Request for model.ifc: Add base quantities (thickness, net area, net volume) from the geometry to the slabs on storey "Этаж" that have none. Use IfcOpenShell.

First a look at what the model holds.

```python
import ifcopenshell
import ifcopenshell.util.element
import ifcopenshell.util.unit

model = ifcopenshell.open("model.ifc")
print(model.schema)
for unit_type in ("LENGTHUNIT", "AREAUNIT", "VOLUMEUNIT"):
    print(unit_type, ifcopenshell.util.unit.calculate_unit_scale(model, unit_type))
storey = next(s for s in model.by_type("IfcBuildingStorey") if s.Name == "Этаж")
slabs = [e for e in ifcopenshell.util.element.get_decomposition(storey) if e.is_a("IfcSlab")]
for e in sorted(slabs, key=lambda e: e.id()):
    print(e.id(), e.is_a(), e.Name, list(ifcopenshell.util.element.get_psets(e, qtos_only=True)), sep=" | ")
```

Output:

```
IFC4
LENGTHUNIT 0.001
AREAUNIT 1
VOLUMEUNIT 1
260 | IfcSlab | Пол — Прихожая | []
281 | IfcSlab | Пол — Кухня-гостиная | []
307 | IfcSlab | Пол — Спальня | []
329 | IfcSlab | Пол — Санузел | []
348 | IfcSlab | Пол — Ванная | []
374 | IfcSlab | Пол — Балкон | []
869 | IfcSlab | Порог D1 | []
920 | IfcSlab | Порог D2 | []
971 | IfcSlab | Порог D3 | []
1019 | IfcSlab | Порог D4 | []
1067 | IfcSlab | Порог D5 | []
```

```python
import ifcopenshell
import ifcopenshell.api.pset
import ifcopenshell.geom
import ifcopenshell.util.element
import ifcopenshell.util.shape
import ifcopenshell.util.unit

model = ifcopenshell.open("model.ifc")
unit_scale = ifcopenshell.util.unit.calculate_unit_scale(model)
area_scale = ifcopenshell.util.unit.calculate_unit_scale(model, "AREAUNIT")
volume_scale = ifcopenshell.util.unit.calculate_unit_scale(model, "VOLUMEUNIT")
settings = ifcopenshell.geom.settings()

storey = next(s for s in model.by_type("IfcBuildingStorey") if s.Name == "Этаж")
slabs = [e for e in ifcopenshell.util.element.get_decomposition(storey) if e.is_a("IfcSlab")]

for e in sorted(slabs, key=lambda e: e.id()):
    if ifcopenshell.util.element.get_psets(e, qtos_only=True, should_inherit=False):
        continue
    # Geometry comes back in metres, in the element's own axes.
    shape = ifcopenshell.geom.create_shape(settings, e)
    values = {
        "Width": ifcopenshell.util.shape.get_z(shape.geometry) / unit_scale,
        "NetArea": ifcopenshell.util.shape.get_footprint_area(shape.geometry) / area_scale,
        "NetVolume": ifcopenshell.util.shape.get_volume(shape.geometry) / volume_scale,
    }
    qto = ifcopenshell.api.pset.add_qto(model, product=e, name="Qto_SlabBaseQuantities")
    ifcopenshell.api.pset.edit_qto(model, qto=qto, properties=values)
    print(e.id(), {k: round(v, 3) for k, v in values.items()})

model.write("model_updated.ifc")
```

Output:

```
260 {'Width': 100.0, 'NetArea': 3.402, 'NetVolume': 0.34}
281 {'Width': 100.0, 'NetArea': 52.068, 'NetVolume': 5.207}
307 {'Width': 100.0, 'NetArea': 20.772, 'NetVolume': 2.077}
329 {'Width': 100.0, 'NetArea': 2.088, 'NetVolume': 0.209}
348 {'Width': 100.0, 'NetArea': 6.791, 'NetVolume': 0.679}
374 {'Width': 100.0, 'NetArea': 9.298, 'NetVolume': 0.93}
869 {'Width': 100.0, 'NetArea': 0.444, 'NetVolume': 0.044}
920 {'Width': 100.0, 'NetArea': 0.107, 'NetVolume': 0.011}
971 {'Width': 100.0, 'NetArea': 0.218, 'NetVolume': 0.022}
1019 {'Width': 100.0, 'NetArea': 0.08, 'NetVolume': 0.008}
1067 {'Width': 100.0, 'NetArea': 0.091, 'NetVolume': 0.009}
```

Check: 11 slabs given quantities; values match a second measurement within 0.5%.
